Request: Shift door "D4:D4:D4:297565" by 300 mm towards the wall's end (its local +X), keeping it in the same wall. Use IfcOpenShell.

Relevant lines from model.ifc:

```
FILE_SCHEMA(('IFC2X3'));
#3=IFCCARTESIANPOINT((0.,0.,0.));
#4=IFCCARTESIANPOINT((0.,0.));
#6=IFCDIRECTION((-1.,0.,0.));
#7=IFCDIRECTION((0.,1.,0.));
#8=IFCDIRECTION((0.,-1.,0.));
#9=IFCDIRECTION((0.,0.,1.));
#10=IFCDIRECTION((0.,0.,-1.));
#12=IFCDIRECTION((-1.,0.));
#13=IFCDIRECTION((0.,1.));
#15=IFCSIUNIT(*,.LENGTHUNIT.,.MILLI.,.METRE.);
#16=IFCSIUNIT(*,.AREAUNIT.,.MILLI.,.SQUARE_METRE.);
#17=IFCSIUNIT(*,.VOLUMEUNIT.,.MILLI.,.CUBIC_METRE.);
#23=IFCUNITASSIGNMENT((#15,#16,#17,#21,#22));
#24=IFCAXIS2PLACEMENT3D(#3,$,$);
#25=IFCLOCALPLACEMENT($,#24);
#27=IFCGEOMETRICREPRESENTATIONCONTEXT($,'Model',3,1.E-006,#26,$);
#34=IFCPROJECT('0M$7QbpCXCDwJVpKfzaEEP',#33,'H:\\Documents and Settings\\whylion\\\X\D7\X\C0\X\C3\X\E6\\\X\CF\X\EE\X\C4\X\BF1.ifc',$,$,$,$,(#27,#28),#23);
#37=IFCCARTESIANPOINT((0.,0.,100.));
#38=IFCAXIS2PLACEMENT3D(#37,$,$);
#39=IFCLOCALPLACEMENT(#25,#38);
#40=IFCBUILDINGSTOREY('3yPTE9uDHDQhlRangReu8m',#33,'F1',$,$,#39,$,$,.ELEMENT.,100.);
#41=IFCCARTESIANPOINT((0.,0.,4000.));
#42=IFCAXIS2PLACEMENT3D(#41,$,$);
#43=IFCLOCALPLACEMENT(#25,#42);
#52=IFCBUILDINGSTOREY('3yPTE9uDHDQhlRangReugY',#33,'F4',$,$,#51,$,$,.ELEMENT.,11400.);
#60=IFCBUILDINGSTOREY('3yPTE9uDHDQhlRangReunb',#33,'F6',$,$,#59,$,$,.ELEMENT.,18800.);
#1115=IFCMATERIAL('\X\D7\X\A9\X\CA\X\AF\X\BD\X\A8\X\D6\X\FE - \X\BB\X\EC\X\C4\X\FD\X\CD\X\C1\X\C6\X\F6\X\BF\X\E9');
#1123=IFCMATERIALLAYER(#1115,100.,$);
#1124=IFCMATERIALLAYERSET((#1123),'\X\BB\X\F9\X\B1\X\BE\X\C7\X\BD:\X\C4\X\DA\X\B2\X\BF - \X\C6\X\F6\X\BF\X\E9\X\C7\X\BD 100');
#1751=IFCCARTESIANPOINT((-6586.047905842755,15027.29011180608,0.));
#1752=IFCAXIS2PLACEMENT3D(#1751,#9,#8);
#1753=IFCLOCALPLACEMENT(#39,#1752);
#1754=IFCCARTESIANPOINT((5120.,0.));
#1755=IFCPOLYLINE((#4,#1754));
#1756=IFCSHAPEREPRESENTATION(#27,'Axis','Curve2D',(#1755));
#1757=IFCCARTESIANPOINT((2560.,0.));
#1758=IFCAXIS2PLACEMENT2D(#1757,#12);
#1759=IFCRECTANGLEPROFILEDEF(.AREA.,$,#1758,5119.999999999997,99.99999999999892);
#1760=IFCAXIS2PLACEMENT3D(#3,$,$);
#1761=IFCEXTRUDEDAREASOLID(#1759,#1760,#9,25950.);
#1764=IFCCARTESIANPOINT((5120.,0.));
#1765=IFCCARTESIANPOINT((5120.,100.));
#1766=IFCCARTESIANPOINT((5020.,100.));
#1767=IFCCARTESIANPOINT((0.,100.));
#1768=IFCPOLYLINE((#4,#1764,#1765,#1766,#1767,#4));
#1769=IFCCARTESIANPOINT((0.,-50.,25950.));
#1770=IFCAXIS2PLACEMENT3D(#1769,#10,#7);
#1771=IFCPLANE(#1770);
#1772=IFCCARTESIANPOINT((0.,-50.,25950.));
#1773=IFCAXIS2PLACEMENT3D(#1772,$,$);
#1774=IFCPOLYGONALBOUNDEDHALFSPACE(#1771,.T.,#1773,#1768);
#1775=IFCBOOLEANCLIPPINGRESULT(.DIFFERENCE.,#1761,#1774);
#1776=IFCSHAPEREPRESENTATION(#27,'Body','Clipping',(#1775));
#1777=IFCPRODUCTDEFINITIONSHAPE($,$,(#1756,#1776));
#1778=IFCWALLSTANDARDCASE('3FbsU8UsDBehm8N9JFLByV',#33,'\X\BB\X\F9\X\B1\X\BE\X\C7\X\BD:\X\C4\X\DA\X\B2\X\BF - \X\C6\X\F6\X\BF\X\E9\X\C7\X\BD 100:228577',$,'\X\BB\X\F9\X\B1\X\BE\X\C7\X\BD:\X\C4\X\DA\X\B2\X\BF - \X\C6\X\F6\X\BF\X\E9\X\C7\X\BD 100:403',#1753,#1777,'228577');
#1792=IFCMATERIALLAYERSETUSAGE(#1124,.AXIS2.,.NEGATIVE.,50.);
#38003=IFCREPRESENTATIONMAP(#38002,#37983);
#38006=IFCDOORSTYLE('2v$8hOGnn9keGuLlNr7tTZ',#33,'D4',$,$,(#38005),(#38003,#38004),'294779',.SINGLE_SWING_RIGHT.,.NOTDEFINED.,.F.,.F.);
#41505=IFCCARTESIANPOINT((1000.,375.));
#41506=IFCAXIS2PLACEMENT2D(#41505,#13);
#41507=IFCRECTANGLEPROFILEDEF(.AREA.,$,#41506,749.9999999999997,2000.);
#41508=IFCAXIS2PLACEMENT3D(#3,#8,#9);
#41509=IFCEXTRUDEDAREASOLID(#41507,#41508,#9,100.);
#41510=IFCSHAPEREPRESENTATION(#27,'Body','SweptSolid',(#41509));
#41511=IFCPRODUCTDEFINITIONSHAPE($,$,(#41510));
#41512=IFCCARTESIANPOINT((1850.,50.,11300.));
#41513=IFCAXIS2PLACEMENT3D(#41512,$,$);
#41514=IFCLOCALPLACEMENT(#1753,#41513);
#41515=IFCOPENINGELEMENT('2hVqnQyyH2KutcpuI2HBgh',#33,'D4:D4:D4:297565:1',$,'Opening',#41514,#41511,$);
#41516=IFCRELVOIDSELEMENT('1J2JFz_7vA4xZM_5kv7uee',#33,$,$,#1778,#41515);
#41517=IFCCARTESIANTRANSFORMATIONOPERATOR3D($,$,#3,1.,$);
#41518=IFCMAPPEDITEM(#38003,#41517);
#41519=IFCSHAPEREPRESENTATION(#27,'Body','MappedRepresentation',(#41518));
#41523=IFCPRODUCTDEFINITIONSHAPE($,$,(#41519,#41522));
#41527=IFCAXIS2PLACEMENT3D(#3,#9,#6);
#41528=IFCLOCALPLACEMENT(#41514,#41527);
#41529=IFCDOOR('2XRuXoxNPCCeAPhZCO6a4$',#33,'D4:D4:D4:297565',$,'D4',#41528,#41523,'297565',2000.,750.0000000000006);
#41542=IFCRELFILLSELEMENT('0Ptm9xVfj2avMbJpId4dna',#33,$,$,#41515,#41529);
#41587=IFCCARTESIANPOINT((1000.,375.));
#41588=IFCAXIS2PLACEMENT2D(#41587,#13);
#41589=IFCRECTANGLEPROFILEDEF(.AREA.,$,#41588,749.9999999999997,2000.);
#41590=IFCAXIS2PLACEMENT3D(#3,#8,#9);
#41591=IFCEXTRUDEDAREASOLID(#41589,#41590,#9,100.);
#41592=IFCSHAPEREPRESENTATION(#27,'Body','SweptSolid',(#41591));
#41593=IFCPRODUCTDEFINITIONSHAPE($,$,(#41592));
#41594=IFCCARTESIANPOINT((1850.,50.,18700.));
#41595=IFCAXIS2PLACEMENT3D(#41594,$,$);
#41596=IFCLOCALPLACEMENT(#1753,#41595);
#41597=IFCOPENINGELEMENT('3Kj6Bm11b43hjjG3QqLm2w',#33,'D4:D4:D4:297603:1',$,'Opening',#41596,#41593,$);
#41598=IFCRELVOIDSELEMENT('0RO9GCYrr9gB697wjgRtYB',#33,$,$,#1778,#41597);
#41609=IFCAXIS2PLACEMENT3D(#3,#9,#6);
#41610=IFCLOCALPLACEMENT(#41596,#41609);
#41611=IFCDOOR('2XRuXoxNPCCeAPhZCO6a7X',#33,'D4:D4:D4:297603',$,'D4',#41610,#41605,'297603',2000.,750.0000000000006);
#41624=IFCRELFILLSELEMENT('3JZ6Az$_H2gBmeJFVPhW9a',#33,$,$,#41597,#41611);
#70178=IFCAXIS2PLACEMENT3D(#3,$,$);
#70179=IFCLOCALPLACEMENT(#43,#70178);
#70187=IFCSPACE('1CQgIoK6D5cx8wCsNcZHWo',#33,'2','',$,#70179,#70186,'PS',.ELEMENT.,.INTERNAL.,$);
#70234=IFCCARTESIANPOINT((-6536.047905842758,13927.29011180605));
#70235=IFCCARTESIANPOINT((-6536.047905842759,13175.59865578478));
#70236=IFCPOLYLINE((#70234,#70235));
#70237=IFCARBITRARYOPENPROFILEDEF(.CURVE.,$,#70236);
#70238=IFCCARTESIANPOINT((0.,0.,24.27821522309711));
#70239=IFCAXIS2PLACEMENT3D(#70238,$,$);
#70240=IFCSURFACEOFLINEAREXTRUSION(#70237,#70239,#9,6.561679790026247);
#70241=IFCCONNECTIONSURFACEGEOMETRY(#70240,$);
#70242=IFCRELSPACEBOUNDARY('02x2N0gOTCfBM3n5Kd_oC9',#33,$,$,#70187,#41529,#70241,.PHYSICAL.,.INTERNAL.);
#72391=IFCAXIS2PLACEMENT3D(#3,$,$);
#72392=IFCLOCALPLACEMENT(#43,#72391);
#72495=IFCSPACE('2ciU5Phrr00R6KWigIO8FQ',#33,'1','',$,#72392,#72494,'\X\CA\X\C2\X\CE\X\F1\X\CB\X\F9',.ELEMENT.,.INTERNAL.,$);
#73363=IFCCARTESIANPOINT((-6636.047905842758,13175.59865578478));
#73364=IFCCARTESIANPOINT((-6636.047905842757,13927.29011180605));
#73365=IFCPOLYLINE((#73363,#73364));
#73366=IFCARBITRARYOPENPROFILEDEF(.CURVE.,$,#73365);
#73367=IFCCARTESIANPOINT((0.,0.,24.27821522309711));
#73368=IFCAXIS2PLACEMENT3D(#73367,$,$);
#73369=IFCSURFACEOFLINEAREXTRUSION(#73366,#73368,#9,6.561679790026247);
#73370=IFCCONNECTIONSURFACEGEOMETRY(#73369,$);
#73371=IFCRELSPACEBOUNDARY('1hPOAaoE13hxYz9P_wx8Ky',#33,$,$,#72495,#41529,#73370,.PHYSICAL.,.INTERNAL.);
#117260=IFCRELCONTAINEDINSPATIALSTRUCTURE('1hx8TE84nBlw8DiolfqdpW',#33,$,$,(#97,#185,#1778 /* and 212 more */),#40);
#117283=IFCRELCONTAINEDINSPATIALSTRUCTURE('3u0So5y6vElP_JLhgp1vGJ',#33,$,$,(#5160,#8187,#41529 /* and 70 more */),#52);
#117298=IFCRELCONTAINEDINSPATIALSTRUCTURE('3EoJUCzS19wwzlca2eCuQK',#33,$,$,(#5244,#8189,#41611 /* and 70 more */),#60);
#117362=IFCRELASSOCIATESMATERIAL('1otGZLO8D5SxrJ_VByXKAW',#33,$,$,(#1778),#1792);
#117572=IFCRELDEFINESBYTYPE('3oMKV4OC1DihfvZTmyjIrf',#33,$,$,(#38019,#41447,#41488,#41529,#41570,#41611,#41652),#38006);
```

```python
import numpy as np
import ifcopenshell
import ifcopenshell.api.geometry
import ifcopenshell.util.placement
import ifcopenshell.util.unit

model = ifcopenshell.open("model.ifc")
unit_scale = ifcopenshell.util.unit.calculate_unit_scale(model)

door = model.by_id(41529)
opening = door.FillsVoids[0].RelatingOpeningElement
wall = opening.VoidsElements[0].RelatingBuildingElement

wall_matrix = ifcopenshell.util.placement.get_local_placement(wall.ObjectPlacement)
shift = wall_matrix[:3, 0] * 0.3 / unit_scale
before = ifcopenshell.util.placement.get_local_placement(door.ObjectPlacement)[:3, 3].copy()

# The door is placed relative to its opening, so it follows when the opening moves.
matrix = ifcopenshell.util.placement.get_local_placement(opening.ObjectPlacement)
matrix[:3, 3] += shift
ifcopenshell.api.geometry.edit_object_placement(
    model, product=opening, matrix=matrix, is_si=False, should_transform_children=True
)

# Space boundary surfaces are stored in each space's coordinates; move them too.
for rel in door.ProvidesBoundaries:
    if not rel.ConnectionGeometry:
        continue
    surface = rel.ConnectionGeometry.SurfaceOnRelatingElement
    space_matrix = ifcopenshell.util.placement.get_local_placement(rel.RelatingSpace.ObjectPlacement)
    point = np.array(surface.Position.Location.Coordinates) + space_matrix[:3, :3].T @ shift
    surface.Position = model.createIfcAxis2Placement3D(
        model.createIfcCartesianPoint(point.tolist()), surface.Position.Axis, surface.Position.RefDirection
    )

after = ifcopenshell.util.placement.get_local_placement(door.ObjectPlacement)[:3, 3]
print("door moved by", (after - before).round(3) + 0.0)

model.write("model_updated.ifc")
```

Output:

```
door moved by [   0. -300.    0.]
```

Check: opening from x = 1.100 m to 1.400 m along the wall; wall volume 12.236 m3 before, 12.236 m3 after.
